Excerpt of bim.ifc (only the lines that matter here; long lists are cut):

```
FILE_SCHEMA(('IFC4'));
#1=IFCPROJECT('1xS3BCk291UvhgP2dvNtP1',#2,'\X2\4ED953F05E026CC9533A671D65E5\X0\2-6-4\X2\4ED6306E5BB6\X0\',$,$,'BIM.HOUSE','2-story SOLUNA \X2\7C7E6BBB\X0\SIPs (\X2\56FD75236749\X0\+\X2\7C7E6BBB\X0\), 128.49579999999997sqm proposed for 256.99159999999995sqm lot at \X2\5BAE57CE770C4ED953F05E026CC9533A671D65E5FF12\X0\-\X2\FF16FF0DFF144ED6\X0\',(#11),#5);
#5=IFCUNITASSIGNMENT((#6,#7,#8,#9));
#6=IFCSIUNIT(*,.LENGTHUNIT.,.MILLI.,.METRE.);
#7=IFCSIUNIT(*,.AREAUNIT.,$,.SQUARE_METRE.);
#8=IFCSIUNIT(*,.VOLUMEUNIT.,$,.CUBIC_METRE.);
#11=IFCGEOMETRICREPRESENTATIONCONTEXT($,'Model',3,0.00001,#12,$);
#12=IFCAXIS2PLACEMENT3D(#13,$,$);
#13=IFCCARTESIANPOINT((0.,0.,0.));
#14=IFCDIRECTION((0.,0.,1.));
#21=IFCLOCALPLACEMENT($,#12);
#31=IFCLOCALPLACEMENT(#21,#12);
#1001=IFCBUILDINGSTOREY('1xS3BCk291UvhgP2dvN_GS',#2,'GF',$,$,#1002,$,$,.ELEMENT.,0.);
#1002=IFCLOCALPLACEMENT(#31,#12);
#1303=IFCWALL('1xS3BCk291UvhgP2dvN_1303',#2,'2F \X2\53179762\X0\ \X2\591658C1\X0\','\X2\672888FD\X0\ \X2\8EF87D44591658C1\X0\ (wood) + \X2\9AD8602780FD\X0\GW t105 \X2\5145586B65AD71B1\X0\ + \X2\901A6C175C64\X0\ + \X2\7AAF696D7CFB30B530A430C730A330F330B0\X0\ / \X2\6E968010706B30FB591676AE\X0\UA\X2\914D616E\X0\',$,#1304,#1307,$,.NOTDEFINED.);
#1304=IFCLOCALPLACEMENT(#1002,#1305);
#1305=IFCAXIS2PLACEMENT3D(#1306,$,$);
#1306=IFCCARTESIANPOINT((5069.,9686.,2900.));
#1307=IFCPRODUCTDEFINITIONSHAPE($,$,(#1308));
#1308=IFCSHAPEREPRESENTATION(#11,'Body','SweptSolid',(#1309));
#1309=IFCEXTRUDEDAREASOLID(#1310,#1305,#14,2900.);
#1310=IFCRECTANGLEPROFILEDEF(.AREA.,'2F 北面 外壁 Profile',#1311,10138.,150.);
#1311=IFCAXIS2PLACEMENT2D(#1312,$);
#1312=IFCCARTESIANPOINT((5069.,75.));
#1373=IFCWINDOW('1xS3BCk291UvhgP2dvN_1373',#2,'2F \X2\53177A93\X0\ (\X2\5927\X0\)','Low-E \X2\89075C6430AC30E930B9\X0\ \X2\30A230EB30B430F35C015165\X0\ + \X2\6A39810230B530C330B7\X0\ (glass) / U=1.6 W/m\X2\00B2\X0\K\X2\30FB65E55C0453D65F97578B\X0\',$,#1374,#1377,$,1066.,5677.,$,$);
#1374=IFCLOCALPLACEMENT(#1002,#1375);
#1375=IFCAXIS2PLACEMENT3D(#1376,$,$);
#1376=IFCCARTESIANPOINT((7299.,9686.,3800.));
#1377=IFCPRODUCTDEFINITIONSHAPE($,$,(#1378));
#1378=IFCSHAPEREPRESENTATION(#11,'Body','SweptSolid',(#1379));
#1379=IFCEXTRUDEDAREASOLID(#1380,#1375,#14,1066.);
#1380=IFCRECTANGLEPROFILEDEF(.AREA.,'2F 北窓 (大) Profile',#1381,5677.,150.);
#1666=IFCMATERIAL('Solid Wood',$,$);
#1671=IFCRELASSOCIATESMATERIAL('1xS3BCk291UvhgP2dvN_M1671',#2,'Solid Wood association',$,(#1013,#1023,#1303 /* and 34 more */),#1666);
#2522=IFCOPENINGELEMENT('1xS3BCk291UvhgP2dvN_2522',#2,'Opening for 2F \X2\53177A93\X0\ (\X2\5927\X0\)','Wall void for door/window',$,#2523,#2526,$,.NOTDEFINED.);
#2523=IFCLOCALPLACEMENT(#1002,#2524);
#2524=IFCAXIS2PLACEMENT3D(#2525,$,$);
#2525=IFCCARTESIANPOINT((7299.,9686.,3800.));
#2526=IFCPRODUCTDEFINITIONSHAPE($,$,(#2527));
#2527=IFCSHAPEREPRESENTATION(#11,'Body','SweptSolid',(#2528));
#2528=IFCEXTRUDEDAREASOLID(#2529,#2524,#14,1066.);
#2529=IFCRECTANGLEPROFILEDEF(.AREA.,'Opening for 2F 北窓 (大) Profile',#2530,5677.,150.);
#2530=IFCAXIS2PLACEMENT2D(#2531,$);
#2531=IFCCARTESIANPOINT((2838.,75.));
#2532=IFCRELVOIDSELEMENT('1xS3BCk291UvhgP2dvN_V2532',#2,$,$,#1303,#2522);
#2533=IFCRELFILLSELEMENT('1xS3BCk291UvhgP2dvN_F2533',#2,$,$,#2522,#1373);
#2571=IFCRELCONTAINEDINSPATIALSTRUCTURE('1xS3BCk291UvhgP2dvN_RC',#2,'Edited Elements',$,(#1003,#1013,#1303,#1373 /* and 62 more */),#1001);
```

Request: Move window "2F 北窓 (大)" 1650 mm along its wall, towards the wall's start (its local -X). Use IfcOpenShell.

```python
import ifcopenshell
import ifcopenshell.api.geometry
import ifcopenshell.util.placement
import ifcopenshell.util.unit

model = ifcopenshell.open("bim.ifc")
unit_scale = ifcopenshell.util.unit.calculate_unit_scale(model)

window = model.by_guid("1xS3BCk291UvhgP2dvN_1373")
opening = window.FillsVoids[0].RelatingOpeningElement
wall = opening.VoidsElements[0].RelatingBuildingElement

wall_matrix = ifcopenshell.util.placement.get_local_placement(wall.ObjectPlacement)
shift = wall_matrix[:3, 0] * -1.65 / unit_scale
before = ifcopenshell.util.placement.get_local_placement(window.ObjectPlacement)[:3, 3].copy()

# The window is not placed relative to its opening, so move both.
for product in (opening, window):
    matrix = ifcopenshell.util.placement.get_local_placement(product.ObjectPlacement)
    matrix[:3, 3] += shift
    ifcopenshell.api.geometry.edit_object_placement(model, product=product, matrix=matrix, is_si=False)

after = ifcopenshell.util.placement.get_local_placement(window.ObjectPlacement)[:3, 3]
print("window moved by", (after - before).round(3) + 0.0)

model.write("bim_edited.ifc")
```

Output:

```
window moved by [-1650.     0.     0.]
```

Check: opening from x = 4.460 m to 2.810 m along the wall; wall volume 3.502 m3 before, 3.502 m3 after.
